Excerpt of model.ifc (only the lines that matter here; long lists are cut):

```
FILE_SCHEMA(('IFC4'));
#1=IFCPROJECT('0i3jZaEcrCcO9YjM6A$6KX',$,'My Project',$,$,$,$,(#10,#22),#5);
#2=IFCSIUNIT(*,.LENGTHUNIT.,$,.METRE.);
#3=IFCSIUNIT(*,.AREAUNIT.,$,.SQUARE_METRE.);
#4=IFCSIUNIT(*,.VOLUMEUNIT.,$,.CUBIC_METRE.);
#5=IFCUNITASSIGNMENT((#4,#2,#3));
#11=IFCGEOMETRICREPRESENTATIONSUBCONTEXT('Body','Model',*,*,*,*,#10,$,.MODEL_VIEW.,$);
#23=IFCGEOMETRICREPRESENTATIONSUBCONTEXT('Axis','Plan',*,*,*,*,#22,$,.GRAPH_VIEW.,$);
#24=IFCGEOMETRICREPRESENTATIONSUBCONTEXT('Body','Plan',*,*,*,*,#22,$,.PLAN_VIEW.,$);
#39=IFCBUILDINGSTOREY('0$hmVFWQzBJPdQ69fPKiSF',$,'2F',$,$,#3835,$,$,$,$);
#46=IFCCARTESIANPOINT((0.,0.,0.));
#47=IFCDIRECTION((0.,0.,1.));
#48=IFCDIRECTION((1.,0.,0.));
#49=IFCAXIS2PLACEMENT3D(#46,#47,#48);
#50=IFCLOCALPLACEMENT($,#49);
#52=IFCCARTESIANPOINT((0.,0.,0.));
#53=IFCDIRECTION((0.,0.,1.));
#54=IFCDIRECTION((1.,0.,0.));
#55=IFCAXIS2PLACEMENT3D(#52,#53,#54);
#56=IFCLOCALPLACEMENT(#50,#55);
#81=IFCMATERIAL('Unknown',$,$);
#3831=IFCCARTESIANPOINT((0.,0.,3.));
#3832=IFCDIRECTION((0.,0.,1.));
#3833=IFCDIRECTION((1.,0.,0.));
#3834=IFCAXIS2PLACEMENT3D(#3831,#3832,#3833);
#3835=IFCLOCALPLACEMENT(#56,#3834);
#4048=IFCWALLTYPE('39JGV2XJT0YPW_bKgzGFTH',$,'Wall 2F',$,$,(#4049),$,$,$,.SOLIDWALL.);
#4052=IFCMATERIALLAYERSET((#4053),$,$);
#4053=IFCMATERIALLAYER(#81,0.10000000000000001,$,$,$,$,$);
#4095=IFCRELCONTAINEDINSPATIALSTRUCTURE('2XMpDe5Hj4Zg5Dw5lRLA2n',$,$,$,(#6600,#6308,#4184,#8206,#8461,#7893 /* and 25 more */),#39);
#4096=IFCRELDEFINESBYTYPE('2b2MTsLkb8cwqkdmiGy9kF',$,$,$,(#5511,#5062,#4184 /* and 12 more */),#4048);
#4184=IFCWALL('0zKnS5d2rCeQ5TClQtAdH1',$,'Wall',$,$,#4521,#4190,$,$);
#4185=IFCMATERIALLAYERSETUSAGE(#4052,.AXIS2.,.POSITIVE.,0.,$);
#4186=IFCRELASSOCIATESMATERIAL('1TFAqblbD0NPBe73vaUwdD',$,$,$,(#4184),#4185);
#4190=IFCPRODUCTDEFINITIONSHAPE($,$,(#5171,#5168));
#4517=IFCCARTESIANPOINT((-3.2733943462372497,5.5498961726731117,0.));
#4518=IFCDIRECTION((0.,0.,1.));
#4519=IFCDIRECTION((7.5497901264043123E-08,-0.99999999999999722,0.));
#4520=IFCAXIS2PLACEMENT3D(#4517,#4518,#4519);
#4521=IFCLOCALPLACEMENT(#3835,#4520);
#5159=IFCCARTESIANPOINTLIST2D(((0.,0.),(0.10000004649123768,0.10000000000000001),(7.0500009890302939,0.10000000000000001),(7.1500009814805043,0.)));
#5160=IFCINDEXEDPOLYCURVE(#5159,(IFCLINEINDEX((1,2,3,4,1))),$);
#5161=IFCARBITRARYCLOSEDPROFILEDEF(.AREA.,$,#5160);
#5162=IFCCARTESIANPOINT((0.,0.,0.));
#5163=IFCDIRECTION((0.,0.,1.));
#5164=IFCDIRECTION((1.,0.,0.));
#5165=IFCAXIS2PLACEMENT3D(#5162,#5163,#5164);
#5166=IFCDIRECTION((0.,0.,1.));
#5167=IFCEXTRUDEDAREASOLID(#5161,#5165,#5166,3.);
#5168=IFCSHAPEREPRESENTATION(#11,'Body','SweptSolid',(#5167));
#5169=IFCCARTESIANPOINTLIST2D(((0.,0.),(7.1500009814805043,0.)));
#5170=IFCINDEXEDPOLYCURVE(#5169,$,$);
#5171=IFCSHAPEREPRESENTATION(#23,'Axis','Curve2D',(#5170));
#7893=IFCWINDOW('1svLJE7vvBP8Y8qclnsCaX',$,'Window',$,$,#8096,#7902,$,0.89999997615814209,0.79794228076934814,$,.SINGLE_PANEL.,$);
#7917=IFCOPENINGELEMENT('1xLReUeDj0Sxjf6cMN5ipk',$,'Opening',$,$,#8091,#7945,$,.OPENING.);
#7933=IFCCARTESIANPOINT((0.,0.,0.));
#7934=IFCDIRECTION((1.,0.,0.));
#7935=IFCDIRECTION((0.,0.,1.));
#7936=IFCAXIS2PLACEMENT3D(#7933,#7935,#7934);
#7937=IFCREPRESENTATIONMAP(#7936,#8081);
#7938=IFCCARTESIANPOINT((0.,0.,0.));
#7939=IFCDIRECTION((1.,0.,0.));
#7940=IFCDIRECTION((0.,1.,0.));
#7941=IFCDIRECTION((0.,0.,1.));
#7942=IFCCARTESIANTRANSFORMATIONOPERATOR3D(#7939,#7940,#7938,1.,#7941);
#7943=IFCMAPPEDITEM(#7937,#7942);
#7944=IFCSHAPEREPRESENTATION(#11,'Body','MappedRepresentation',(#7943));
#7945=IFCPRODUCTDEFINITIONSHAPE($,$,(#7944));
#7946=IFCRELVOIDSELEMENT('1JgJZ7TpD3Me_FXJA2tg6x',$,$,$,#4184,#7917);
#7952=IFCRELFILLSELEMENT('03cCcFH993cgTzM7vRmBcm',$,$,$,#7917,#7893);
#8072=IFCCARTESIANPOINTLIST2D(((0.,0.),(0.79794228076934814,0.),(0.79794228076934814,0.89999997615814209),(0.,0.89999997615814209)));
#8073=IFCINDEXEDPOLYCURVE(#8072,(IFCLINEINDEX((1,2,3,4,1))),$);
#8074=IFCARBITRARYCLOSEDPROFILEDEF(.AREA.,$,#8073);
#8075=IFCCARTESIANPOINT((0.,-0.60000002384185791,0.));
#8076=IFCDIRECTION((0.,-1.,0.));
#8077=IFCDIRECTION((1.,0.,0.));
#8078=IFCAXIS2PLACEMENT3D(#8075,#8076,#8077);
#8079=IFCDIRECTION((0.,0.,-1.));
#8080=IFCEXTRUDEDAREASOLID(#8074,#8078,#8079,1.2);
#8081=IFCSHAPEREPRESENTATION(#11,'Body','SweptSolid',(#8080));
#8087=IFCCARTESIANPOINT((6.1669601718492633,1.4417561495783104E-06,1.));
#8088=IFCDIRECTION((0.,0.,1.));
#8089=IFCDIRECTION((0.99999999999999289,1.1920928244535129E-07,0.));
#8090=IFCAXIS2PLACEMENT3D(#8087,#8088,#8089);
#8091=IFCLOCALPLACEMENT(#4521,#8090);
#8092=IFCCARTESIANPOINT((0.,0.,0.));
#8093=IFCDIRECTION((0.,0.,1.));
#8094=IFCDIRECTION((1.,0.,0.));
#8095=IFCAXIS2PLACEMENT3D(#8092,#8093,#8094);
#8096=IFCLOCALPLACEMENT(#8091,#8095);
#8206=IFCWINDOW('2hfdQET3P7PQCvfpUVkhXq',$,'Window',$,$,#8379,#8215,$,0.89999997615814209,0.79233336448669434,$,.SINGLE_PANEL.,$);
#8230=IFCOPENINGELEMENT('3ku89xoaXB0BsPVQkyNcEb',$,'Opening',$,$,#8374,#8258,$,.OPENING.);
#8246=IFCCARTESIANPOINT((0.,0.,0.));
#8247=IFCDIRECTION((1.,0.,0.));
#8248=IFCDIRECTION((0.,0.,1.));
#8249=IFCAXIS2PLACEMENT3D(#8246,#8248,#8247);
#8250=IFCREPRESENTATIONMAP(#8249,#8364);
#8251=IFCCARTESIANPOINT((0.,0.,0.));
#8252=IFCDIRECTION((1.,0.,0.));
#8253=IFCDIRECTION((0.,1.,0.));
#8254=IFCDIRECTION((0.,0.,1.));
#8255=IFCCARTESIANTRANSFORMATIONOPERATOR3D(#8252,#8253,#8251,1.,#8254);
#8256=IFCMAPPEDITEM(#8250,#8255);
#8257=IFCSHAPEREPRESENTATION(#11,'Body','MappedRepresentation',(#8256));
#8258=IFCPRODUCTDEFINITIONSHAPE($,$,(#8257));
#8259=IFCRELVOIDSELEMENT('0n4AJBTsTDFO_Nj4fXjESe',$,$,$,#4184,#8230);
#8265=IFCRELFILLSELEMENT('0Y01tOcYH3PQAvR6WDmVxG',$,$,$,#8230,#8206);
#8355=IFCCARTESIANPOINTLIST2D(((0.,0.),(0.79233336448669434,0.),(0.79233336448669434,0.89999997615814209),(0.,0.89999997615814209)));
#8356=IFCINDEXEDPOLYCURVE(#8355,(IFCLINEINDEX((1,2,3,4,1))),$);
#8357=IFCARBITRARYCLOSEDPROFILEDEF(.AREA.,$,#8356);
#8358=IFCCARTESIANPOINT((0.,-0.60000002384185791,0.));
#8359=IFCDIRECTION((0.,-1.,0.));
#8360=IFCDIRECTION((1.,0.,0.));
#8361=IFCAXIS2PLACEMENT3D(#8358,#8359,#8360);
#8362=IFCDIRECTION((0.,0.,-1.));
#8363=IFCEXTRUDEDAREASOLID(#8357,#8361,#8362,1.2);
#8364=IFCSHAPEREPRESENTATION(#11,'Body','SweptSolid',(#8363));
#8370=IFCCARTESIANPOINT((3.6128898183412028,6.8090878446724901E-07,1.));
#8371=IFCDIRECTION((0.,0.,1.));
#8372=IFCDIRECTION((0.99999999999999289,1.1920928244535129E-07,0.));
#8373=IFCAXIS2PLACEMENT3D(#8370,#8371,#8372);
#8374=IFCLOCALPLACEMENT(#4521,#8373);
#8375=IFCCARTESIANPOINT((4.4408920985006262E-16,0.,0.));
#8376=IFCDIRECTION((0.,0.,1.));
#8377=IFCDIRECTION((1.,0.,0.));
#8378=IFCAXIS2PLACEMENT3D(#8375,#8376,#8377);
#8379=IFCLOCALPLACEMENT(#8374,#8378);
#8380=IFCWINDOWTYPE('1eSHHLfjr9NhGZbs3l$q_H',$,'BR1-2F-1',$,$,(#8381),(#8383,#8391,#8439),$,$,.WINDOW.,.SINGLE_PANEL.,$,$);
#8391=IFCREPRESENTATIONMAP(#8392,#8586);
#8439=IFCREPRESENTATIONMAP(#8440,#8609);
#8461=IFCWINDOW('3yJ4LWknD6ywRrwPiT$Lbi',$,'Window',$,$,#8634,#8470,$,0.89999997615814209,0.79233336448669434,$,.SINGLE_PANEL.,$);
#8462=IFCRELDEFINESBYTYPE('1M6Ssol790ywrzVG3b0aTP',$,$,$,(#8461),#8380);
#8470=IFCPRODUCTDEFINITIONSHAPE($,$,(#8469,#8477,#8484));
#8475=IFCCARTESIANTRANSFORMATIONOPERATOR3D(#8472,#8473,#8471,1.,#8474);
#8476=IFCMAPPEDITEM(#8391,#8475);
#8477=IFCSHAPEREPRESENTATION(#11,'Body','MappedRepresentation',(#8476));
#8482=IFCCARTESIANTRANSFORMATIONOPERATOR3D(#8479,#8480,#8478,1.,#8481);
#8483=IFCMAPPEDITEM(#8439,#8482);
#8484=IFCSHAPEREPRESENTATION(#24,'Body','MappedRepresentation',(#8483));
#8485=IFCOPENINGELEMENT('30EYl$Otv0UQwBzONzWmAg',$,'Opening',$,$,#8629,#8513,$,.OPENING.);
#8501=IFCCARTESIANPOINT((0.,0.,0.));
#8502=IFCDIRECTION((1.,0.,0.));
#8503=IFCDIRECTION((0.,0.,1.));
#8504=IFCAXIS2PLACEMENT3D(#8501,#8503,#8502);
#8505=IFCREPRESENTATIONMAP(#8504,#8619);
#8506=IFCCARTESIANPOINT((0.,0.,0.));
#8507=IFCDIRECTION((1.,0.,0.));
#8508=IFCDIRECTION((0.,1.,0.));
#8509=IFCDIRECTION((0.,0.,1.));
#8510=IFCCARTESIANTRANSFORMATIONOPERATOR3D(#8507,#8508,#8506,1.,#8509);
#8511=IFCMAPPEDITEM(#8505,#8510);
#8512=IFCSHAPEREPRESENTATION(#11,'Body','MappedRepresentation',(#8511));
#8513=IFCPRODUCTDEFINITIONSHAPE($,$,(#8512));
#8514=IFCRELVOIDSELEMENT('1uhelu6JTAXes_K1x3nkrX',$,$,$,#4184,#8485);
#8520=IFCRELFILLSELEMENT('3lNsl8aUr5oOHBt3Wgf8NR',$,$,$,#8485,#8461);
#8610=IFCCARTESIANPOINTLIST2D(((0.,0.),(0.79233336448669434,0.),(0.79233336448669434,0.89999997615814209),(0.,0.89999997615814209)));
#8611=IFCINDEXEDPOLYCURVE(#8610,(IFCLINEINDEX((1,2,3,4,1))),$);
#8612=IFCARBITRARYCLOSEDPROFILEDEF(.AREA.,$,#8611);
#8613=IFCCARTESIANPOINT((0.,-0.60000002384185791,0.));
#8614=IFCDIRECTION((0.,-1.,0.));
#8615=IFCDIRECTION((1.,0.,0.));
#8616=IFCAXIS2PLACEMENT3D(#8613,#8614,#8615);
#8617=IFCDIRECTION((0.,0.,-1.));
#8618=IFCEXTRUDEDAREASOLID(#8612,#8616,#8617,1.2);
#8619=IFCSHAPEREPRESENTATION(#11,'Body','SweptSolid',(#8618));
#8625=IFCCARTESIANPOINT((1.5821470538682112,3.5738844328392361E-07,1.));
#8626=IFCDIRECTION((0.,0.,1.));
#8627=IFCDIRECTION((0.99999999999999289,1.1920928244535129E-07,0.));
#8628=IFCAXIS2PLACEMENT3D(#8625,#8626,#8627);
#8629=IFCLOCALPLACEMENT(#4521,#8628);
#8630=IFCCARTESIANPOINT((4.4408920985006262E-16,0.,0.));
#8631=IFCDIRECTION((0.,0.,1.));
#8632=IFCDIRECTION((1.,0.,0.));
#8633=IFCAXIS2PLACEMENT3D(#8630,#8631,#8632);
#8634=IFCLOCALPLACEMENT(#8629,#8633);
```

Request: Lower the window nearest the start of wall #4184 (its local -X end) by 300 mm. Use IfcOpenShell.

```python
import numpy as np
import ifcopenshell
import ifcopenshell.api.geometry
import ifcopenshell.util.placement
import ifcopenshell.util.unit

model = ifcopenshell.open("model.ifc")
unit_scale = ifcopenshell.util.unit.calculate_unit_scale(model)

window = model.by_guid("3yJ4LWknD6ywRrwPiT$Lbi")
opening = window.FillsVoids[0].RelatingOpeningElement
dz = -0.3

shift = np.array([0.0, 0.0, dz])
# The window is placed relative to its opening, so it follows when the opening moves.
matrix = ifcopenshell.util.placement.get_local_placement(opening.ObjectPlacement)
matrix[:3, 3] += shift
ifcopenshell.api.geometry.edit_object_placement(
    model, product=opening, matrix=matrix, is_si=False, should_transform_children=True
)

print(f"moved by {dz * unit_scale:+.3f} m")

model.write("model_v2.ifc")
```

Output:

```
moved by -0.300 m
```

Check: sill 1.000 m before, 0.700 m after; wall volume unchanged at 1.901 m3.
